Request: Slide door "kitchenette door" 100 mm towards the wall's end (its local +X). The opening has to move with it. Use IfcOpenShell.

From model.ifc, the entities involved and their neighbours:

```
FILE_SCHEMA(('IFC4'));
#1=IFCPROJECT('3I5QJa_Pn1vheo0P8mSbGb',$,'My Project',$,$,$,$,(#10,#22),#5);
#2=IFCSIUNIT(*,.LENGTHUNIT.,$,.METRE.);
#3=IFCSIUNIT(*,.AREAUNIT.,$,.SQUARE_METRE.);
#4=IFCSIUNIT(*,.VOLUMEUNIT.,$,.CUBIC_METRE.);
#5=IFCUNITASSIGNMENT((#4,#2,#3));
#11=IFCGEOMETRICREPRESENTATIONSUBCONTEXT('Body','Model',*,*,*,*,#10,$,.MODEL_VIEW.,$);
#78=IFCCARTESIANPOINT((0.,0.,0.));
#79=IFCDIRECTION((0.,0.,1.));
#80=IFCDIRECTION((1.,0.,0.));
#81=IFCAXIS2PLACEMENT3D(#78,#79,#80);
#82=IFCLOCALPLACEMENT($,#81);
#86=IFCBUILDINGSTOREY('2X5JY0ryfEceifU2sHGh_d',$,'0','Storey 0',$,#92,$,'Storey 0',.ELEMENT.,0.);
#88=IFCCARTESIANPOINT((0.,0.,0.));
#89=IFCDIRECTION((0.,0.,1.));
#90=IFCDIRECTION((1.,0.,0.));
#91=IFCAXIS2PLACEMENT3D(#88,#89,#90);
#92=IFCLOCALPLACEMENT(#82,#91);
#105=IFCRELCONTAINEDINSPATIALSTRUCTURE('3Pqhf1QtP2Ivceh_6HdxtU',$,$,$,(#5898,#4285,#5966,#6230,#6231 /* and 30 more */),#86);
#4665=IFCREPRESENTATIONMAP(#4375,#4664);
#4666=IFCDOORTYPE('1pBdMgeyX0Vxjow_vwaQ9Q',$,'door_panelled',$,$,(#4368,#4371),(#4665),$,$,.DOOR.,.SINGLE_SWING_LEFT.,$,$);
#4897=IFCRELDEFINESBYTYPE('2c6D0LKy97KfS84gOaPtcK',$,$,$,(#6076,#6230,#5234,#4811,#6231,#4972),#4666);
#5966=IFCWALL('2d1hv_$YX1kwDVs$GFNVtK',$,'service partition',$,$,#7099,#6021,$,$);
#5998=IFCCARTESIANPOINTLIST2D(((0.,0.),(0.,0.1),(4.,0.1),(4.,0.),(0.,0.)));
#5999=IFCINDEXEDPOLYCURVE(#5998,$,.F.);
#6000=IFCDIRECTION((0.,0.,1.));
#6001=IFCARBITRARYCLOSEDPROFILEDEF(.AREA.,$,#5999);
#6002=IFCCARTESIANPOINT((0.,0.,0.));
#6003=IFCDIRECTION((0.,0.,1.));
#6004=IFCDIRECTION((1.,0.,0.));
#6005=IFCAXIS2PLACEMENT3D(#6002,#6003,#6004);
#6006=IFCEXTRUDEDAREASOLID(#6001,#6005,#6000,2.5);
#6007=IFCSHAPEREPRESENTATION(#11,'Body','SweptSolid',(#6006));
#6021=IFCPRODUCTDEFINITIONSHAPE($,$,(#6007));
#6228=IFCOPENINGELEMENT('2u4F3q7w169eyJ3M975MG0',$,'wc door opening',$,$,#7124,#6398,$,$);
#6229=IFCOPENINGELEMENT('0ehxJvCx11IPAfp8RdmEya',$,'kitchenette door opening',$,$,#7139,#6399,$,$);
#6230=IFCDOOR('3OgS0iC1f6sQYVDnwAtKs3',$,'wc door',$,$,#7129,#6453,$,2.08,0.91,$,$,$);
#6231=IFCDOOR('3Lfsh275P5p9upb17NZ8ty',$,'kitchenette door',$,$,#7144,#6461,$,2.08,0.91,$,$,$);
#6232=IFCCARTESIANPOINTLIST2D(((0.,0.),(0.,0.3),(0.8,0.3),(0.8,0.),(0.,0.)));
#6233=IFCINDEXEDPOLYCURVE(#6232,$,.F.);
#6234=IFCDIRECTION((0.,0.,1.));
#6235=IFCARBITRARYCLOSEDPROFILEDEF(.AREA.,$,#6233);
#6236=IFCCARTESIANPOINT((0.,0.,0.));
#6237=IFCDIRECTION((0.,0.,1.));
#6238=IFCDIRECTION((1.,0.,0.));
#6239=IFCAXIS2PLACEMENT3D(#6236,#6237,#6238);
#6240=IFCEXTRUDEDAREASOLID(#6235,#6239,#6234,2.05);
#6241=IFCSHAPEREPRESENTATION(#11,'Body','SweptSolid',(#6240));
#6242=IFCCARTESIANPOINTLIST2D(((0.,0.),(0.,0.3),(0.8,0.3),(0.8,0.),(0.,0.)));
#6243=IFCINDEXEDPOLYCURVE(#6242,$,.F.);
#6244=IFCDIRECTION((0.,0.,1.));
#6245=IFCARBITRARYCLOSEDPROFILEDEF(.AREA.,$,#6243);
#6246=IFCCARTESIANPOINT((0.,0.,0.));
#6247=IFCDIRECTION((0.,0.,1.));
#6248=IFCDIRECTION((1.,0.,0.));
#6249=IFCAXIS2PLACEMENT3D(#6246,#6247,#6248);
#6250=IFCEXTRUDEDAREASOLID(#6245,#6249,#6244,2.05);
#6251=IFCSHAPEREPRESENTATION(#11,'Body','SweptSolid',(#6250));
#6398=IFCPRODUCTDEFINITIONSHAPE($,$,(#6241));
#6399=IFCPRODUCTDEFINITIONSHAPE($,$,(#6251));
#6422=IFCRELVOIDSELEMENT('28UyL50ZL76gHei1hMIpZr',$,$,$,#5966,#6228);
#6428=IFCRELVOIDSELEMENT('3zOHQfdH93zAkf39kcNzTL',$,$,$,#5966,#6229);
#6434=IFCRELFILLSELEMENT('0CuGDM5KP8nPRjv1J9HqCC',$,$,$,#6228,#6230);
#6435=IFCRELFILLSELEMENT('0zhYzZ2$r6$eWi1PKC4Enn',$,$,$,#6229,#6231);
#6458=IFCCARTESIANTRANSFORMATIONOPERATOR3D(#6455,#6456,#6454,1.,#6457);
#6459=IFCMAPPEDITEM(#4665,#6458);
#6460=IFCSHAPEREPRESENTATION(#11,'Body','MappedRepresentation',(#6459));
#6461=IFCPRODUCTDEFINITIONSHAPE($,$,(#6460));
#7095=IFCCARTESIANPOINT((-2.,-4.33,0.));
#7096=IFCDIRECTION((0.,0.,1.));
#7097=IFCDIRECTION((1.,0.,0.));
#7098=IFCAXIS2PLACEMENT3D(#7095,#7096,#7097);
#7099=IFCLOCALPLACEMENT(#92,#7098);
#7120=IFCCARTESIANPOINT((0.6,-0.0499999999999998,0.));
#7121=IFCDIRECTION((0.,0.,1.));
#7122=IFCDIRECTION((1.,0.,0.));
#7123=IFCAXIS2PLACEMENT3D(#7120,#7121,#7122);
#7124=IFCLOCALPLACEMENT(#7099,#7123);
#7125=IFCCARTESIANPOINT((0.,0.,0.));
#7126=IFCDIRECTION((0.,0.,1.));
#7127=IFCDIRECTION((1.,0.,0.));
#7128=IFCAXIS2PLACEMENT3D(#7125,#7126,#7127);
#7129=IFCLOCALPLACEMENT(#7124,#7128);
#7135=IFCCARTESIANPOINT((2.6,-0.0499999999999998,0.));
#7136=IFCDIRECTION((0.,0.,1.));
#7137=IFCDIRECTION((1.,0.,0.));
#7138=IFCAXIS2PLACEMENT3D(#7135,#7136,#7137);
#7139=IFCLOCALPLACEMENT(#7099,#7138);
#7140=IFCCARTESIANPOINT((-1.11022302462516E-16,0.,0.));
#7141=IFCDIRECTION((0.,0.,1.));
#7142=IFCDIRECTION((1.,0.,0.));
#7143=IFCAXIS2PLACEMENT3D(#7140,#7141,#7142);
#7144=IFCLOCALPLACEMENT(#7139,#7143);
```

```python
import ifcopenshell
import ifcopenshell.api.geometry
import ifcopenshell.util.placement
import ifcopenshell.util.unit

model = ifcopenshell.open("model.ifc")
unit_scale = ifcopenshell.util.unit.calculate_unit_scale(model)

door = model.by_id(6231)
opening = door.FillsVoids[0].RelatingOpeningElement
wall = opening.VoidsElements[0].RelatingBuildingElement

wall_matrix = ifcopenshell.util.placement.get_local_placement(wall.ObjectPlacement)
shift = wall_matrix[:3, 0] * 0.1 / unit_scale
before = ifcopenshell.util.placement.get_local_placement(door.ObjectPlacement)[:3, 3].copy()

# The door is placed relative to its opening, so it follows when the opening moves.
matrix = ifcopenshell.util.placement.get_local_placement(opening.ObjectPlacement)
matrix[:3, 3] += shift
ifcopenshell.api.geometry.edit_object_placement(
    model, product=opening, matrix=matrix, is_si=False, should_transform_children=True
)

after = ifcopenshell.util.placement.get_local_placement(door.ObjectPlacement)[:3, 3]
print("door moved by", (after - before).round(3) + 0.0)

model.write("model_v2.ifc")
```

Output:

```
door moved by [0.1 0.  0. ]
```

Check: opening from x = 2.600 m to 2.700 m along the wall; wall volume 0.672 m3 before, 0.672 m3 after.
